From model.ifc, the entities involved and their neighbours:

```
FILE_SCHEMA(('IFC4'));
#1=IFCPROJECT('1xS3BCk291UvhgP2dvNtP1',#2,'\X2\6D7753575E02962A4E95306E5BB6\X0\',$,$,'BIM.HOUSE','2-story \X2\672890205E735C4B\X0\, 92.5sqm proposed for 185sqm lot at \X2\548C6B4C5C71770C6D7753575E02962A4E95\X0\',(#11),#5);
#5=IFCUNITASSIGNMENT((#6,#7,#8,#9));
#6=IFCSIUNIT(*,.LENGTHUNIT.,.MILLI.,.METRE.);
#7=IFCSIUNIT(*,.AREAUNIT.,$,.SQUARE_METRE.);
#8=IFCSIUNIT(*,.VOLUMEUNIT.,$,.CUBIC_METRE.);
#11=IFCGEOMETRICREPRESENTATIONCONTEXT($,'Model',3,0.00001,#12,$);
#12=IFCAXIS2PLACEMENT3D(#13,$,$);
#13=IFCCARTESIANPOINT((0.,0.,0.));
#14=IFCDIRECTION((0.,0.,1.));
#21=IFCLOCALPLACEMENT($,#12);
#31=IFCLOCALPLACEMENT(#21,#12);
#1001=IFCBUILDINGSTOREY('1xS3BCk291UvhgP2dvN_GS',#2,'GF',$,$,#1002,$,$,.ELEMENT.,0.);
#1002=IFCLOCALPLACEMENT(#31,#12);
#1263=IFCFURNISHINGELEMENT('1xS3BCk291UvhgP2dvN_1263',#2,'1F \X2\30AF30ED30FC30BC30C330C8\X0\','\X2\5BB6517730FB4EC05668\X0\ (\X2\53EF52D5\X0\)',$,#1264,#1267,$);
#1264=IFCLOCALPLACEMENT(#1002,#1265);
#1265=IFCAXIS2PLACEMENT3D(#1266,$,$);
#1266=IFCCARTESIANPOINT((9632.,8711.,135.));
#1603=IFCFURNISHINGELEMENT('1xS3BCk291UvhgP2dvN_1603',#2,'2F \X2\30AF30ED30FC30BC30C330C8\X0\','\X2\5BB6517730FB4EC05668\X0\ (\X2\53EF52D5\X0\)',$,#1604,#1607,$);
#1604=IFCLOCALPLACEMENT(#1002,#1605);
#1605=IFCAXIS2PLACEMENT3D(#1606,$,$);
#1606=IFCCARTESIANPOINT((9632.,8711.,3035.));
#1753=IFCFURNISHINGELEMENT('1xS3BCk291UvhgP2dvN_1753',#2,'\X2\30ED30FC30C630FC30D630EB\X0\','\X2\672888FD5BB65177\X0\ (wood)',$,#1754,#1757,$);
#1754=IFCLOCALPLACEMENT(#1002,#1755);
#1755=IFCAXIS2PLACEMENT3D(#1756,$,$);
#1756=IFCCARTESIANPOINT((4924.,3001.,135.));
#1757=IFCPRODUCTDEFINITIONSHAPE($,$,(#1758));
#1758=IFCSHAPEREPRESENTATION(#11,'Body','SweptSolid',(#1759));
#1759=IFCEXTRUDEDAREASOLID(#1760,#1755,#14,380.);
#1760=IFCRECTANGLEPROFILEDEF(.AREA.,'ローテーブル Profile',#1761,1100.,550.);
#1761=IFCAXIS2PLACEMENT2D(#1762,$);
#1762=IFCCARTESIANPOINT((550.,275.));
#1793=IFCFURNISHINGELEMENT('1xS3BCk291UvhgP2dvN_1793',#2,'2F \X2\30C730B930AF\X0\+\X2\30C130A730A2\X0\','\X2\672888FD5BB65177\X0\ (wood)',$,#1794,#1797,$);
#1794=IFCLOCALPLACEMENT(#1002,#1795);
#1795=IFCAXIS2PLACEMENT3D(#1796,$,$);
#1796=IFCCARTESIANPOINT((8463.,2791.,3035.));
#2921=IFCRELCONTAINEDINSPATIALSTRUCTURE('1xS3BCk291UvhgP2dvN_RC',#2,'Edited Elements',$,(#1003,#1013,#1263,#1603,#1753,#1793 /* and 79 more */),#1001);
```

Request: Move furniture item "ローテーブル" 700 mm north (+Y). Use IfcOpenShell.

```python
import ifcopenshell
import ifcopenshell.api.geometry
import ifcopenshell.util.placement
import ifcopenshell.util.unit

model = ifcopenshell.open("model.ifc")
unit_scale = ifcopenshell.util.unit.calculate_unit_scale(model)

item = model.by_guid("1xS3BCk291UvhgP2dvN_1753")
matrix = ifcopenshell.util.placement.get_local_placement(item.ObjectPlacement)
matrix[1, 3] += 0.7 / unit_scale
ifcopenshell.api.geometry.edit_object_placement(model, product=item, matrix=matrix, is_si=False)

print(ifcopenshell.util.placement.get_local_placement(item.ObjectPlacement).round(3) + 0.0)

model.write("model_rev.ifc")
```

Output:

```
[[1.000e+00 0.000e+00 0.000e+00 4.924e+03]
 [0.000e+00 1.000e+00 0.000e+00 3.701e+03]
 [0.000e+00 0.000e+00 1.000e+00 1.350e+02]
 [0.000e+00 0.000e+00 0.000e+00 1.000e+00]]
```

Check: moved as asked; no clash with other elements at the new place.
